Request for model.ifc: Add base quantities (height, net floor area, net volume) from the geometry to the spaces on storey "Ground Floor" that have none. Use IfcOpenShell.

First a look at what the model holds.

```python
import ifcopenshell
import ifcopenshell.util.element
import ifcopenshell.util.unit

model = ifcopenshell.open("model.ifc")
print(model.schema)
for unit_type in ("LENGTHUNIT", "AREAUNIT", "VOLUMEUNIT"):
    print(unit_type, ifcopenshell.util.unit.calculate_unit_scale(model, unit_type))
storey = next(s for s in model.by_type("IfcBuildingStorey") if s.Name == "Ground Floor")
spaces = [e for e in ifcopenshell.util.element.get_decomposition(storey) if e.is_a("IfcSpace")]
for e in sorted(spaces, key=lambda e: e.id()):
    print(e.id(), e.is_a(), e.Name, list(ifcopenshell.util.element.get_psets(e, qtos_only=True)), sep=" | ")
```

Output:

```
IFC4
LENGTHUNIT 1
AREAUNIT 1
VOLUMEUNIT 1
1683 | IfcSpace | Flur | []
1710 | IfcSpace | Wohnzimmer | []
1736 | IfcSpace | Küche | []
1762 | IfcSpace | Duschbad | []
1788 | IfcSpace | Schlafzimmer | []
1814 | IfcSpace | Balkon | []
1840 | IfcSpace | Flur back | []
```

```python
import ifcopenshell
import ifcopenshell.api.pset
import ifcopenshell.geom
import ifcopenshell.util.element
import ifcopenshell.util.shape
import ifcopenshell.util.unit

model = ifcopenshell.open("model.ifc")
unit_scale = ifcopenshell.util.unit.calculate_unit_scale(model)
area_scale = ifcopenshell.util.unit.calculate_unit_scale(model, "AREAUNIT")
volume_scale = ifcopenshell.util.unit.calculate_unit_scale(model, "VOLUMEUNIT")
settings = ifcopenshell.geom.settings()

storey = next(s for s in model.by_type("IfcBuildingStorey") if s.Name == "Ground Floor")
spaces = [e for e in ifcopenshell.util.element.get_decomposition(storey) if e.is_a("IfcSpace")]

for e in sorted(spaces, key=lambda e: e.id()):
    if ifcopenshell.util.element.get_psets(e, qtos_only=True, should_inherit=False):
        continue
    # Geometry comes back in metres, in the element's own axes.
    shape = ifcopenshell.geom.create_shape(settings, e)
    values = {
        "Height": ifcopenshell.util.shape.get_z(shape.geometry) / unit_scale,
        "NetFloorArea": ifcopenshell.util.shape.get_footprint_area(shape.geometry) / area_scale,
        "NetVolume": ifcopenshell.util.shape.get_volume(shape.geometry) / volume_scale,
    }
    qto = ifcopenshell.api.pset.add_qto(model, product=e, name="Qto_SpaceBaseQuantities")
    ifcopenshell.api.pset.edit_qto(model, qto=qto, properties=values)
    print(e.id(), {k: round(v, 3) for k, v in values.items()})

model.write("model_v2.ifc")
```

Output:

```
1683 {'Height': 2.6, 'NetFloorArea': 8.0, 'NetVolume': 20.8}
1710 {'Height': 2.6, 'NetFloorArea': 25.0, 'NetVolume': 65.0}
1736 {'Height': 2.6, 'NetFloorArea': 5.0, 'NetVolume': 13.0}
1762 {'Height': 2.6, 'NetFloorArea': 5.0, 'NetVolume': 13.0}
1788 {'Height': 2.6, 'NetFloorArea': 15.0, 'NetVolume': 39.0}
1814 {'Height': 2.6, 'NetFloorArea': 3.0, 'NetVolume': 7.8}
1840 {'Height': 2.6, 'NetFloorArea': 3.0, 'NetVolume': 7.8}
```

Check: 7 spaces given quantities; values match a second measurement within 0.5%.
